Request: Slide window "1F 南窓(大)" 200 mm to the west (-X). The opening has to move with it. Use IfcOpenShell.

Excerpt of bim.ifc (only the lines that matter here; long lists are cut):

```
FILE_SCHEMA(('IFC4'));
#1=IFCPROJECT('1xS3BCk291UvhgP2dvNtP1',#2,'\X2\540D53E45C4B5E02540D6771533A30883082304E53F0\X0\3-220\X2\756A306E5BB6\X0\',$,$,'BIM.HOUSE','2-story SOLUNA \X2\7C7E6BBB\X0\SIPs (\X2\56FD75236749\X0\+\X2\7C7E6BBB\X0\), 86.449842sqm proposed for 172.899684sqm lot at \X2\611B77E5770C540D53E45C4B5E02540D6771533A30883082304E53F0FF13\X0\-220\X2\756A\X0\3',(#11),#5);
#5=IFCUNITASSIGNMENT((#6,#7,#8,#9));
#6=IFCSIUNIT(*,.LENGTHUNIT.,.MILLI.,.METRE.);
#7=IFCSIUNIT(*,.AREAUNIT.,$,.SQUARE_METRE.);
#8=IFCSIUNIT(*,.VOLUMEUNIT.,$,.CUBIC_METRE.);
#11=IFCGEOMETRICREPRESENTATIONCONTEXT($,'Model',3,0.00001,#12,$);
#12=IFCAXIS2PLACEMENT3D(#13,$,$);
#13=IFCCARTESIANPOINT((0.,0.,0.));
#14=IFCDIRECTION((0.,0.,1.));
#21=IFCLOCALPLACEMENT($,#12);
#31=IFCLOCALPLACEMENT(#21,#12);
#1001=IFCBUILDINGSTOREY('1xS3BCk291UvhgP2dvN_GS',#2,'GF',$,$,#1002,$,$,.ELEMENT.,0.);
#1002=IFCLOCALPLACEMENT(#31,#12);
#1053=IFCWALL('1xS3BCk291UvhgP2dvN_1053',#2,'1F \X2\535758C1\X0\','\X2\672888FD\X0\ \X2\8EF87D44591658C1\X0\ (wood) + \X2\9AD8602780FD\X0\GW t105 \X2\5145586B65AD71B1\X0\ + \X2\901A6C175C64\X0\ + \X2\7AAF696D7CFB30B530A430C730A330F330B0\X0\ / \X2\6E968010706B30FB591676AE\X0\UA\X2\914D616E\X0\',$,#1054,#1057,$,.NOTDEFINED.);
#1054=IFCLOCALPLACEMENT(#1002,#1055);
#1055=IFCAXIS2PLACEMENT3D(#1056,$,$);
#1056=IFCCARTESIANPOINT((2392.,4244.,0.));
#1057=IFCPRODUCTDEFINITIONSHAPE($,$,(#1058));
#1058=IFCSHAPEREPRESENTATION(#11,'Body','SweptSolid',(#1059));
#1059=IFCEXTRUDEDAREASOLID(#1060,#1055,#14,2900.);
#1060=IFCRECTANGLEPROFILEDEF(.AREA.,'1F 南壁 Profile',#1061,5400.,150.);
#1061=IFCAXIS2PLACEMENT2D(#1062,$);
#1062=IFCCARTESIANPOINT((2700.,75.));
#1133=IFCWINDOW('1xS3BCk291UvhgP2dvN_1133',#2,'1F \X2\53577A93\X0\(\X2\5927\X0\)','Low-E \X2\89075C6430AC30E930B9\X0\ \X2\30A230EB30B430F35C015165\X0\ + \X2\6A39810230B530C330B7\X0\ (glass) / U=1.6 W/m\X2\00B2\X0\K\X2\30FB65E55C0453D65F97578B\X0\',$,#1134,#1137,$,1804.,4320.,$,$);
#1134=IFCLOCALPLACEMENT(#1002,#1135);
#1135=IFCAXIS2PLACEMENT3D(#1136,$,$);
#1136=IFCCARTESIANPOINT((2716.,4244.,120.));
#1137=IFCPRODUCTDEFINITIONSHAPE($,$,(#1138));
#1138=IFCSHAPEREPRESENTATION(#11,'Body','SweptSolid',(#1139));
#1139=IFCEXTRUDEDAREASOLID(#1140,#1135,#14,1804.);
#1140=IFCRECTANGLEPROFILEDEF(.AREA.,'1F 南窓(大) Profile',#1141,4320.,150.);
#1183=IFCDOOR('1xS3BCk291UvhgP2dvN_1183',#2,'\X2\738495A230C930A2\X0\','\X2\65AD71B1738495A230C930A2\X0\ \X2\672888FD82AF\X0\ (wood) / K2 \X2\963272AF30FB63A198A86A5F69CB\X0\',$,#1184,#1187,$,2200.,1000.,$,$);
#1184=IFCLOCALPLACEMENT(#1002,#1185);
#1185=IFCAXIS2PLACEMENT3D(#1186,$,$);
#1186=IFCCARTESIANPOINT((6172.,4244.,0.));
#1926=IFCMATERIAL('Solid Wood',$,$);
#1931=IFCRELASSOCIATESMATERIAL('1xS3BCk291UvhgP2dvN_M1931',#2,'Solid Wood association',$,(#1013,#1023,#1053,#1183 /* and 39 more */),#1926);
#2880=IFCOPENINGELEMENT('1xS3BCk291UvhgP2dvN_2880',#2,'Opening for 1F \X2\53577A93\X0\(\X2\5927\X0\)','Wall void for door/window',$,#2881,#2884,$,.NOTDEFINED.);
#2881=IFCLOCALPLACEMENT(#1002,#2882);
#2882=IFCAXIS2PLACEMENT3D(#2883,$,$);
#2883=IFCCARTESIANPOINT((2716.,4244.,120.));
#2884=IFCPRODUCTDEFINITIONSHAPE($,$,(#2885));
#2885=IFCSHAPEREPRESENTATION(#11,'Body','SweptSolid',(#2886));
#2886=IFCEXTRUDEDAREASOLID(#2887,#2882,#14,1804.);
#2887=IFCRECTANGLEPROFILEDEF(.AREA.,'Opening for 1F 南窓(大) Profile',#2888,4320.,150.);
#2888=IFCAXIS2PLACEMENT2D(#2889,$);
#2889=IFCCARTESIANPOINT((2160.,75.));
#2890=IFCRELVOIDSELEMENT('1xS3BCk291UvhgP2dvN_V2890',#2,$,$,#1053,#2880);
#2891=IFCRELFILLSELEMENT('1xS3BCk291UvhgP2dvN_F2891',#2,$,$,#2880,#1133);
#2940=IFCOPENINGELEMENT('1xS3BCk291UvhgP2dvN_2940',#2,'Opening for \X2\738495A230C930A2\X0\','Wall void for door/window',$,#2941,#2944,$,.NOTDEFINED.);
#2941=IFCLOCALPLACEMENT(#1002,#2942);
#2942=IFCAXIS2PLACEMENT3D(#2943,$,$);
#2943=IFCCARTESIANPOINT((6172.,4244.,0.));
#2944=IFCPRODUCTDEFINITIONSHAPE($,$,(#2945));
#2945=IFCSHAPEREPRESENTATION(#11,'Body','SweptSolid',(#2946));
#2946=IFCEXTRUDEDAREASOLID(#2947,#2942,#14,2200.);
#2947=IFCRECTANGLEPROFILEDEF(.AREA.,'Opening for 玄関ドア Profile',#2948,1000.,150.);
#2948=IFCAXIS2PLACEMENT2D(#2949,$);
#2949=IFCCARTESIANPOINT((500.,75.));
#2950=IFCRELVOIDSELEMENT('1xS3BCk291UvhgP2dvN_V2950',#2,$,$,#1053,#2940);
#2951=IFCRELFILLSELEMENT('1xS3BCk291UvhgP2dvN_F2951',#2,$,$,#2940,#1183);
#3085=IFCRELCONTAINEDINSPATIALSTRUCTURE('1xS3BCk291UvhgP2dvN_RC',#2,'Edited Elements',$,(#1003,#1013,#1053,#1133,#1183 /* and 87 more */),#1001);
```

```python
import ifcopenshell
import ifcopenshell.api.geometry
import ifcopenshell.util.placement

model = ifcopenshell.open("bim.ifc")

window = model.by_id(1133)
opening = window.FillsVoids[0].RelatingOpeningElement
wall = opening.VoidsElements[0].RelatingBuildingElement

wall_matrix = ifcopenshell.util.placement.get_local_placement(wall.ObjectPlacement)
shift = wall_matrix[:3, 0] * -200.0
before = ifcopenshell.util.placement.get_local_placement(window.ObjectPlacement)[:3, 3].copy()

# The window is not placed relative to its opening, so move both.
for product in (opening, window):
    matrix = ifcopenshell.util.placement.get_local_placement(product.ObjectPlacement)
    matrix[:3, 3] += shift
    ifcopenshell.api.geometry.edit_object_placement(model, product=product, matrix=matrix, is_si=False)

after = ifcopenshell.util.placement.get_local_placement(window.ObjectPlacement)[:3, 3]
print("window moved by", (after - before).round(3) + 0.0)

model.write("bim-out.ifc")
```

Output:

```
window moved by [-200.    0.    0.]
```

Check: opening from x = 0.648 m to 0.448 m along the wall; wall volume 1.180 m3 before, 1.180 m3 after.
